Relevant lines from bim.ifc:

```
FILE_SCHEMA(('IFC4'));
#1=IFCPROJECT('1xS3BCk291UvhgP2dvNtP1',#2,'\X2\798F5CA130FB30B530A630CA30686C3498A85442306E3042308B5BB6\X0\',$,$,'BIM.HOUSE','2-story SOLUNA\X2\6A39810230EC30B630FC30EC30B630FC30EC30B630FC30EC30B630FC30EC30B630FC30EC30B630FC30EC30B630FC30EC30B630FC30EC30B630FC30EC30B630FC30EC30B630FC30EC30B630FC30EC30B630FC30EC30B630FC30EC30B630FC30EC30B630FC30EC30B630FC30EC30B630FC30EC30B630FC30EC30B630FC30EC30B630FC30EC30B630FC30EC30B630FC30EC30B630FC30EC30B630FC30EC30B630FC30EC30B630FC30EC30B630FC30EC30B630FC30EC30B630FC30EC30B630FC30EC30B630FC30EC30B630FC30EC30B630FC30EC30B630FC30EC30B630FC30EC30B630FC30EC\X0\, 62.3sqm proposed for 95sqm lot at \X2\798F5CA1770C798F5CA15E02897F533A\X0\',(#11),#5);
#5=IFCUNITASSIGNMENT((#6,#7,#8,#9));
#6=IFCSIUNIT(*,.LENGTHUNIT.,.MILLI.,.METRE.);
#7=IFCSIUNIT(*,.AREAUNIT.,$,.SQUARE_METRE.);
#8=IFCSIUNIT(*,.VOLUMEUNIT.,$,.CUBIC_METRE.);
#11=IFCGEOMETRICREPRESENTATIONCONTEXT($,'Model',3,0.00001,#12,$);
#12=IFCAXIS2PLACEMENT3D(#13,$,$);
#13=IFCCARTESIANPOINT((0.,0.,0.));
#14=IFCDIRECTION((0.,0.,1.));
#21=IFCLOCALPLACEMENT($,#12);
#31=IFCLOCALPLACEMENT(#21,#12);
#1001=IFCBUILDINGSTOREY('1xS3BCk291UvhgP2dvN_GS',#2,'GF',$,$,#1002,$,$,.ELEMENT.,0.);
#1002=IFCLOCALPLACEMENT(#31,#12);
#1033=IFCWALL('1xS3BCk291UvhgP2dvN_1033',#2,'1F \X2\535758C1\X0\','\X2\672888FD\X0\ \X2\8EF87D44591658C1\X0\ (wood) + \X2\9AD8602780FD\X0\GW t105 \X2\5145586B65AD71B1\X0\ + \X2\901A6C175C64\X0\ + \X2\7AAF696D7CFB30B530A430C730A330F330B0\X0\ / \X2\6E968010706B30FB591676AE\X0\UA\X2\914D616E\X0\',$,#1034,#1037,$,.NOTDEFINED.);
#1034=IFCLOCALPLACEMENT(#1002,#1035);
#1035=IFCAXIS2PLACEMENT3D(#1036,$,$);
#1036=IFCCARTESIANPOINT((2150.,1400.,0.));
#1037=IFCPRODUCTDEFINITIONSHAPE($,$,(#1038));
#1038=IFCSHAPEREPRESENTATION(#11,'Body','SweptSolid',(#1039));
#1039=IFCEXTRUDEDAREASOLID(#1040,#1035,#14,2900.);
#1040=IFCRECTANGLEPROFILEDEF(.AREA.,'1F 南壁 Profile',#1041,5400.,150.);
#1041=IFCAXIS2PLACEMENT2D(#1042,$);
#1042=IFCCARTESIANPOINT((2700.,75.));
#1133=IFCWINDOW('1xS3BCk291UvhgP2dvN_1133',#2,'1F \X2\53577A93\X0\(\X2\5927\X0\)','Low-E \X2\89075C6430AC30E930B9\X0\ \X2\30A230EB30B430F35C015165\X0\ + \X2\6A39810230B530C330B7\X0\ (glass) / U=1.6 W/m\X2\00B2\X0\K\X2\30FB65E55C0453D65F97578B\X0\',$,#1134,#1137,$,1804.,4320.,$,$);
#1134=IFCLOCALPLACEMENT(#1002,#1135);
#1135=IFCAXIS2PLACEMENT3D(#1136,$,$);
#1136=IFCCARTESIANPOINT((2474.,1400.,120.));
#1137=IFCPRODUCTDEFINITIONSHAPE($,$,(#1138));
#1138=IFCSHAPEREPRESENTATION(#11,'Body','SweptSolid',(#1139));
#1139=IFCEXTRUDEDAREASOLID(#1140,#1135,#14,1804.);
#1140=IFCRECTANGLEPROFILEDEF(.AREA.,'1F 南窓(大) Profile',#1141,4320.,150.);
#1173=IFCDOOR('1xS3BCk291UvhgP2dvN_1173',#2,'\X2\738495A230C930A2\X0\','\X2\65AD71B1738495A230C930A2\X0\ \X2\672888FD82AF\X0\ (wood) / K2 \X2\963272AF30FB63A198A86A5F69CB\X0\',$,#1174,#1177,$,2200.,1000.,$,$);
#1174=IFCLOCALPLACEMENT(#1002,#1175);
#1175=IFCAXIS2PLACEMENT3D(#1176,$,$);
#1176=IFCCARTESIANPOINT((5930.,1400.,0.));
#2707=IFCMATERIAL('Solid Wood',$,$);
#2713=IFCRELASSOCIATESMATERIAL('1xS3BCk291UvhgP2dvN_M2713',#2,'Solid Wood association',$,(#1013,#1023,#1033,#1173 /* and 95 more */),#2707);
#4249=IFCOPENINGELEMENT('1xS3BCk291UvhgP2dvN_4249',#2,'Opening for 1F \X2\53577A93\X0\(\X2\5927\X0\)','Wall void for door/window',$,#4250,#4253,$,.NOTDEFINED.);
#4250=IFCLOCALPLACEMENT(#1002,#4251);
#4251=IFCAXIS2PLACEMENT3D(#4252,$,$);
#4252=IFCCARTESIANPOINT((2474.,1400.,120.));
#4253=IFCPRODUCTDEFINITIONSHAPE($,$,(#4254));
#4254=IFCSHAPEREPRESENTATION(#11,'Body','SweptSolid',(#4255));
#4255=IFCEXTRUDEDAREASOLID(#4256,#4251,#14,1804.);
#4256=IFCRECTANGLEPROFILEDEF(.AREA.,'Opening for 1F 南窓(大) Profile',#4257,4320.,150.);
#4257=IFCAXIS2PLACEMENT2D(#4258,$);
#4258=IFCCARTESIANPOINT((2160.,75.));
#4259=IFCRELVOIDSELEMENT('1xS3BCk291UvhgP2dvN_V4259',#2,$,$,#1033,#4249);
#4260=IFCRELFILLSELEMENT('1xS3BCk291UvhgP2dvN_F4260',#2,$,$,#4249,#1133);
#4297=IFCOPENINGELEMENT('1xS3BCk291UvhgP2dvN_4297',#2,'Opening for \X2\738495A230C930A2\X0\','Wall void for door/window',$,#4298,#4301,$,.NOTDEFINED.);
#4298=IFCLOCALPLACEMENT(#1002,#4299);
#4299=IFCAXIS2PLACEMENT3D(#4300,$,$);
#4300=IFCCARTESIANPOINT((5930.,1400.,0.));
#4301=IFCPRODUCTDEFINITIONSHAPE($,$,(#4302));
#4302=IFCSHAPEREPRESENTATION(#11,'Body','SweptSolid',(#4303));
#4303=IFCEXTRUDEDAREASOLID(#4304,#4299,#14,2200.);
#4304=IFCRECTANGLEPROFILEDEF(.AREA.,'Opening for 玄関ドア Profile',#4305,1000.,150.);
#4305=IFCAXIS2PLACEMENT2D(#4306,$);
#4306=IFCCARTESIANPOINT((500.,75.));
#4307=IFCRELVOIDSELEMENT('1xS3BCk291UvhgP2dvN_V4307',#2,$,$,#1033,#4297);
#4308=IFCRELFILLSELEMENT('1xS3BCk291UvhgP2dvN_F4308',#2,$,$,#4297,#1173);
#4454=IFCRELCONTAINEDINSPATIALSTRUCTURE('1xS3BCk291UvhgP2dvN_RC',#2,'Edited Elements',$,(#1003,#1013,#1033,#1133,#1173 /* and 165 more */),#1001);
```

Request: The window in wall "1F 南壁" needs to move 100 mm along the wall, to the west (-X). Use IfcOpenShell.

```python
import ifcopenshell
import ifcopenshell.api.geometry
import ifcopenshell.util.placement

model = ifcopenshell.open("bim.ifc")

window = model.by_guid("1xS3BCk291UvhgP2dvN_1133")
opening = window.FillsVoids[0].RelatingOpeningElement
wall = opening.VoidsElements[0].RelatingBuildingElement

wall_matrix = ifcopenshell.util.placement.get_local_placement(wall.ObjectPlacement)
shift = wall_matrix[:3, 0] * -100.0
before = ifcopenshell.util.placement.get_local_placement(window.ObjectPlacement)[:3, 3].copy()

# The window is not placed relative to its opening, so move both.
for product in (opening, window):
    matrix = ifcopenshell.util.placement.get_local_placement(product.ObjectPlacement)
    matrix[:3, 3] += shift
    ifcopenshell.api.geometry.edit_object_placement(model, product=product, matrix=matrix, is_si=False)

after = ifcopenshell.util.placement.get_local_placement(window.ObjectPlacement)[:3, 3]
print("window moved by", (after - before).round(3) + 0.0)

model.write("bim_edited.ifc")
```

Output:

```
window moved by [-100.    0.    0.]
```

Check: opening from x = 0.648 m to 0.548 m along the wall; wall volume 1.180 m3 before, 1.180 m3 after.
